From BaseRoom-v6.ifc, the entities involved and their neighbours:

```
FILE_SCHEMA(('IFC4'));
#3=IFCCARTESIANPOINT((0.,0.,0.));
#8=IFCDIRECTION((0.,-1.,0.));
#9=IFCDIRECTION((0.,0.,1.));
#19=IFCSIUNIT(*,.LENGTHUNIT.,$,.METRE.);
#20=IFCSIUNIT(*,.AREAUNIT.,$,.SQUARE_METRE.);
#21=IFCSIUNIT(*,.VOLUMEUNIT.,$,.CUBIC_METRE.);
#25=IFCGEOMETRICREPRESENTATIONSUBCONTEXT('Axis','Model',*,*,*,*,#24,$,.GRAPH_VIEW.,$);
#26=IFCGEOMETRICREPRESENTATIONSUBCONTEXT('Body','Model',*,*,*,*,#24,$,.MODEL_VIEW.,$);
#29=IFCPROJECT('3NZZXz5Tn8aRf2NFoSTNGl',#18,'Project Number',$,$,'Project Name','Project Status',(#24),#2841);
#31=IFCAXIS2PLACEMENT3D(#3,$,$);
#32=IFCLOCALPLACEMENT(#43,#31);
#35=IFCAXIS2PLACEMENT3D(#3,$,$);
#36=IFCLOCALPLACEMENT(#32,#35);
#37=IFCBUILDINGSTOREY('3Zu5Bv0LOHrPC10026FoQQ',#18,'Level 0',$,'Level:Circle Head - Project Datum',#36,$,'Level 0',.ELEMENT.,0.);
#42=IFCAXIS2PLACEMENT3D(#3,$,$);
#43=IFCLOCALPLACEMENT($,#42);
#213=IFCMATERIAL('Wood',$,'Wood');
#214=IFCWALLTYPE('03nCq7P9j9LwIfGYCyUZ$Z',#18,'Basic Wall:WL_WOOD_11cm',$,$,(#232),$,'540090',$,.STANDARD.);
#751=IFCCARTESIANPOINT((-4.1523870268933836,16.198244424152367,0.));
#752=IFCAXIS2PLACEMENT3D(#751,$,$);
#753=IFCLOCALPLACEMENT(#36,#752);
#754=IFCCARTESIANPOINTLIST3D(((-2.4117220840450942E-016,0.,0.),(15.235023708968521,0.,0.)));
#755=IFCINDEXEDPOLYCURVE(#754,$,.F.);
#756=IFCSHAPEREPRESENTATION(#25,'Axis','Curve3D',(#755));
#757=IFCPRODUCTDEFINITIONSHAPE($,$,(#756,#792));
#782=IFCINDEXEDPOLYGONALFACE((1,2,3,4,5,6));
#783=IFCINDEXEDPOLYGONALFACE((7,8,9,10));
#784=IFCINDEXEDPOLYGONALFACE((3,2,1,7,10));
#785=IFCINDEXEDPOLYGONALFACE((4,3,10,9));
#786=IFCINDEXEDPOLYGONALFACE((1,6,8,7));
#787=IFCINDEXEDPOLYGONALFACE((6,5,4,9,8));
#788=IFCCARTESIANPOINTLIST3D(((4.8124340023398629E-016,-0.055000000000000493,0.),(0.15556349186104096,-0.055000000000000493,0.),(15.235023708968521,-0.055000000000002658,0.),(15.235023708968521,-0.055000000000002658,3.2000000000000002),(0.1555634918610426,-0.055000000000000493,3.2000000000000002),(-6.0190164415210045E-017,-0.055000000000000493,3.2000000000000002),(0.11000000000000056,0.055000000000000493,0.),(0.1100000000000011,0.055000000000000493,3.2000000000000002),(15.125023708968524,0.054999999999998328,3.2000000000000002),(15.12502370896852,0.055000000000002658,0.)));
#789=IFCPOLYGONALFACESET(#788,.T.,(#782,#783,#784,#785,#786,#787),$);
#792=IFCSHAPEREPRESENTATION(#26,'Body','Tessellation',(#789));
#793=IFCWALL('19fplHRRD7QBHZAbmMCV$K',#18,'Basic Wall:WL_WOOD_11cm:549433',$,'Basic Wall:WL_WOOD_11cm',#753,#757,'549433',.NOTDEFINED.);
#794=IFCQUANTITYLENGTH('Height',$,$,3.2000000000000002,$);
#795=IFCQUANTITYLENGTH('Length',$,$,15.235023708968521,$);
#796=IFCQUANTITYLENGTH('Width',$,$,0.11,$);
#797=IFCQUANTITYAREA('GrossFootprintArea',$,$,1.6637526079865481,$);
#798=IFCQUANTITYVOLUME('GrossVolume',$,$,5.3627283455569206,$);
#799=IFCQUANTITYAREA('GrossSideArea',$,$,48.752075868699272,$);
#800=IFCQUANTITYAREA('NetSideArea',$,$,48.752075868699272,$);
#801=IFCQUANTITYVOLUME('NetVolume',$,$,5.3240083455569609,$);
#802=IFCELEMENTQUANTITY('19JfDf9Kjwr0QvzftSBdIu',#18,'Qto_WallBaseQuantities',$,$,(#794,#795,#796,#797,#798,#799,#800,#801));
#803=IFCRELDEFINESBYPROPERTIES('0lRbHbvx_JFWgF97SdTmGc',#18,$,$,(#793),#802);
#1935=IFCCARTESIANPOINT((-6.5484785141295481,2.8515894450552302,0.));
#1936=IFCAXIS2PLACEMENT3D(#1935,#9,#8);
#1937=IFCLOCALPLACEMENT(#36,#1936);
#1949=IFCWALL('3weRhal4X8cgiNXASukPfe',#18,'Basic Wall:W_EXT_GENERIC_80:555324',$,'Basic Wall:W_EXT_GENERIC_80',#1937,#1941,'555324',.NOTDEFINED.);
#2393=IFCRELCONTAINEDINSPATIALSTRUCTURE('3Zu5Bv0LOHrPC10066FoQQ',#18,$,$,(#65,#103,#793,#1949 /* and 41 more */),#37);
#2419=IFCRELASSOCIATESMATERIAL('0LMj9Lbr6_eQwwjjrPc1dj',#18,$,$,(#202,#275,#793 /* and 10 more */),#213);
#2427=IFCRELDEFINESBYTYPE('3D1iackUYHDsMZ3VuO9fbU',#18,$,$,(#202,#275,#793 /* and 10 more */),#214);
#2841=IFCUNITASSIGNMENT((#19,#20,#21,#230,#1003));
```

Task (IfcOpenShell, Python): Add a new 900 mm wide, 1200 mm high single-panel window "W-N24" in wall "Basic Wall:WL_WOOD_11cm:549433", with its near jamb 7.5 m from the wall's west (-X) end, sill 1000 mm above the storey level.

```python
import numpy as np
import ifcopenshell
import ifcopenshell.api.feature
import ifcopenshell.api.geometry
import ifcopenshell.api.pset
import ifcopenshell.api.root
import ifcopenshell.api.spatial
import ifcopenshell.geom
import ifcopenshell.util.element
import ifcopenshell.util.placement
import ifcopenshell.util.representation
import ifcopenshell.util.shape
import ifcopenshell.util.unit

model = ifcopenshell.open("BaseRoom-v6.ifc")
unit_scale = ifcopenshell.util.unit.calculate_unit_scale(model)
area_scale = ifcopenshell.util.unit.calculate_unit_scale(model, "AREAUNIT")
volume_scale = ifcopenshell.util.unit.calculate_unit_scale(model, "VOLUMEUNIT")
settings = ifcopenshell.geom.settings()


def volume(element):
    """Net volume in cubic metres, openings subtracted."""
    shape = ifcopenshell.geom.create_shape(settings, element)
    return ifcopenshell.util.shape.get_volume(shape.geometry)


wall = model.by_guid("19fplHRRD7QBHZAbmMCV$K")
storey = ifcopenshell.util.element.get_container(wall, ifc_class="IfcBuildingStorey")
context = ifcopenshell.util.representation.get_context(model, "Model", "Body", "MODEL_VIEW")
before = volume(wall)

width, height, from_end, sill = 0.9, 1.2, 7.5, 1  # metres

# The wall runs along its own X axis, and the end named is its -X end.
wall_shape = ifcopenshell.geom.create_shape(settings, wall)
x, y, z = ifcopenshell.util.shape.get_vertices(wall_shape.geometry).T
start = x.min() + from_end
face, thickness = float(y.min()), float(y.max() - y.min())
wall_matrix = ifcopenshell.util.placement.get_local_placement(wall.ObjectPlacement)
level = ifcopenshell.util.placement.get_local_placement(storey.ObjectPlacement)[2, 3]


def in_wall(x, y):
    """Placement at x, y metres in the wall's axes, at sill height."""
    matrix = wall_matrix.copy()
    matrix[:, 3] = wall_matrix @ np.array([x / unit_scale, y / unit_scale, 0.0, 1.0])
    matrix[2, 3] = level + sill / unit_scale
    return matrix


# Opening: a box that overshoots both wall faces by 50 mm.
opening = ifcopenshell.api.root.create_entity(model, ifc_class="IfcOpeningElement", predefined_type="OPENING")
box = ifcopenshell.api.geometry.add_wall_representation(
    model, context=context, length=width, height=height, thickness=thickness + 0.1
)
ifcopenshell.api.geometry.assign_representation(model, product=opening, representation=box)
ifcopenshell.api.geometry.edit_object_placement(model, product=opening, matrix=in_wall(start, face - 0.05), is_si=False)
ifcopenshell.api.feature.add_feature(model, feature=opening, element=wall)

window = ifcopenshell.api.root.create_entity(model, ifc_class="IfcWindow", name="W-N24", predefined_type="WINDOW")
window.OverallWidth, window.OverallHeight = width / unit_scale, height / unit_scale
window.PartitioningType = "SINGLE_PANEL"
body = ifcopenshell.api.geometry.add_window_representation(
    model,
    context=context,
    overall_width=window.OverallWidth,
    overall_height=window.OverallHeight,
    partition_type="SINGLE_PANEL",
)
ifcopenshell.api.geometry.assign_representation(model, product=window, representation=body)
ifcopenshell.api.spatial.assign_container(model, products=[window], relating_structure=storey)
ifcopenshell.api.feature.add_filling(model, opening=opening, element=window)

# Centre the window in the wall's thickness.
ifcopenshell.api.geometry.edit_object_placement(model, product=window, matrix=in_wall(start, face), is_si=False)
window_shape = ifcopenshell.geom.create_shape(settings, window)
depth = ifcopenshell.util.shape.get_vertices(window_shape.geometry)[:, 1]
offset = face + thickness / 2 - (depth.min() + depth.max()) / 2
ifcopenshell.api.geometry.edit_object_placement(model, product=window, matrix=in_wall(start, offset), is_si=False)

after = volume(wall)

# Update the wall's stored quantities.
qto = model.by_id(ifcopenshell.util.element.get_pset(wall, "Qto_WallBaseQuantities", should_inherit=False)["id"])
ifcopenshell.api.pset.edit_qto(model, qto=qto, properties={
    "NetSideArea": after / thickness / area_scale,
    "NetVolume": after / volume_scale,
})

print(f"wall volume {before:.3f} -> {after:.3f} m3")

model.write("BaseRoom-v6_updated.ifc")
```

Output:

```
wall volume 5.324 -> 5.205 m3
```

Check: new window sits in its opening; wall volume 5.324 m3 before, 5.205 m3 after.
